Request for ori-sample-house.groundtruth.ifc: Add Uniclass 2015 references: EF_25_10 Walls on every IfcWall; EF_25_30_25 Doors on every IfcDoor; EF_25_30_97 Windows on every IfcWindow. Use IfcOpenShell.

First a look at what the model holds.

```python
import ifcopenshell

model = ifcopenshell.open("ori-sample-house.groundtruth.ifc")
print(model.schema)
print("classifications:", [c.Name for c in model.by_type("IfcClassification")])
for ifc_class in ("IfcDoor", "IfcRoof", "IfcStair", "IfcWall", "IfcWindow"):
    print(ifc_class, len(model.by_type(ifc_class)))
```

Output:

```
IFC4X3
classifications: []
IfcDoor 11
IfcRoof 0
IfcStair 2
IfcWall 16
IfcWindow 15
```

```python
import ifcopenshell
import ifcopenshell.api.classification

model = ifcopenshell.open("ori-sample-house.groundtruth.ifc")

system = ifcopenshell.api.classification.add_classification(model, classification="Uniclass 2015")

codes = {
    "IfcWall": ("EF_25_10", "Walls"),
    "IfcDoor": ("EF_25_30_25", "Doors"),
    "IfcWindow": ("EF_25_30_97", "Windows"),
}
for ifc_class, (code, name) in codes.items():
    products = model.by_type(ifc_class)
    ifcopenshell.api.classification.add_reference(
        model, products=products, classification=system, identification=code, name=name
    )
    print(code, len(products))

model.write("ori-sample-house.groundtruth_rev.ifc")
```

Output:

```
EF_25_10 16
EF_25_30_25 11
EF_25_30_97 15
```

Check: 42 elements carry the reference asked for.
